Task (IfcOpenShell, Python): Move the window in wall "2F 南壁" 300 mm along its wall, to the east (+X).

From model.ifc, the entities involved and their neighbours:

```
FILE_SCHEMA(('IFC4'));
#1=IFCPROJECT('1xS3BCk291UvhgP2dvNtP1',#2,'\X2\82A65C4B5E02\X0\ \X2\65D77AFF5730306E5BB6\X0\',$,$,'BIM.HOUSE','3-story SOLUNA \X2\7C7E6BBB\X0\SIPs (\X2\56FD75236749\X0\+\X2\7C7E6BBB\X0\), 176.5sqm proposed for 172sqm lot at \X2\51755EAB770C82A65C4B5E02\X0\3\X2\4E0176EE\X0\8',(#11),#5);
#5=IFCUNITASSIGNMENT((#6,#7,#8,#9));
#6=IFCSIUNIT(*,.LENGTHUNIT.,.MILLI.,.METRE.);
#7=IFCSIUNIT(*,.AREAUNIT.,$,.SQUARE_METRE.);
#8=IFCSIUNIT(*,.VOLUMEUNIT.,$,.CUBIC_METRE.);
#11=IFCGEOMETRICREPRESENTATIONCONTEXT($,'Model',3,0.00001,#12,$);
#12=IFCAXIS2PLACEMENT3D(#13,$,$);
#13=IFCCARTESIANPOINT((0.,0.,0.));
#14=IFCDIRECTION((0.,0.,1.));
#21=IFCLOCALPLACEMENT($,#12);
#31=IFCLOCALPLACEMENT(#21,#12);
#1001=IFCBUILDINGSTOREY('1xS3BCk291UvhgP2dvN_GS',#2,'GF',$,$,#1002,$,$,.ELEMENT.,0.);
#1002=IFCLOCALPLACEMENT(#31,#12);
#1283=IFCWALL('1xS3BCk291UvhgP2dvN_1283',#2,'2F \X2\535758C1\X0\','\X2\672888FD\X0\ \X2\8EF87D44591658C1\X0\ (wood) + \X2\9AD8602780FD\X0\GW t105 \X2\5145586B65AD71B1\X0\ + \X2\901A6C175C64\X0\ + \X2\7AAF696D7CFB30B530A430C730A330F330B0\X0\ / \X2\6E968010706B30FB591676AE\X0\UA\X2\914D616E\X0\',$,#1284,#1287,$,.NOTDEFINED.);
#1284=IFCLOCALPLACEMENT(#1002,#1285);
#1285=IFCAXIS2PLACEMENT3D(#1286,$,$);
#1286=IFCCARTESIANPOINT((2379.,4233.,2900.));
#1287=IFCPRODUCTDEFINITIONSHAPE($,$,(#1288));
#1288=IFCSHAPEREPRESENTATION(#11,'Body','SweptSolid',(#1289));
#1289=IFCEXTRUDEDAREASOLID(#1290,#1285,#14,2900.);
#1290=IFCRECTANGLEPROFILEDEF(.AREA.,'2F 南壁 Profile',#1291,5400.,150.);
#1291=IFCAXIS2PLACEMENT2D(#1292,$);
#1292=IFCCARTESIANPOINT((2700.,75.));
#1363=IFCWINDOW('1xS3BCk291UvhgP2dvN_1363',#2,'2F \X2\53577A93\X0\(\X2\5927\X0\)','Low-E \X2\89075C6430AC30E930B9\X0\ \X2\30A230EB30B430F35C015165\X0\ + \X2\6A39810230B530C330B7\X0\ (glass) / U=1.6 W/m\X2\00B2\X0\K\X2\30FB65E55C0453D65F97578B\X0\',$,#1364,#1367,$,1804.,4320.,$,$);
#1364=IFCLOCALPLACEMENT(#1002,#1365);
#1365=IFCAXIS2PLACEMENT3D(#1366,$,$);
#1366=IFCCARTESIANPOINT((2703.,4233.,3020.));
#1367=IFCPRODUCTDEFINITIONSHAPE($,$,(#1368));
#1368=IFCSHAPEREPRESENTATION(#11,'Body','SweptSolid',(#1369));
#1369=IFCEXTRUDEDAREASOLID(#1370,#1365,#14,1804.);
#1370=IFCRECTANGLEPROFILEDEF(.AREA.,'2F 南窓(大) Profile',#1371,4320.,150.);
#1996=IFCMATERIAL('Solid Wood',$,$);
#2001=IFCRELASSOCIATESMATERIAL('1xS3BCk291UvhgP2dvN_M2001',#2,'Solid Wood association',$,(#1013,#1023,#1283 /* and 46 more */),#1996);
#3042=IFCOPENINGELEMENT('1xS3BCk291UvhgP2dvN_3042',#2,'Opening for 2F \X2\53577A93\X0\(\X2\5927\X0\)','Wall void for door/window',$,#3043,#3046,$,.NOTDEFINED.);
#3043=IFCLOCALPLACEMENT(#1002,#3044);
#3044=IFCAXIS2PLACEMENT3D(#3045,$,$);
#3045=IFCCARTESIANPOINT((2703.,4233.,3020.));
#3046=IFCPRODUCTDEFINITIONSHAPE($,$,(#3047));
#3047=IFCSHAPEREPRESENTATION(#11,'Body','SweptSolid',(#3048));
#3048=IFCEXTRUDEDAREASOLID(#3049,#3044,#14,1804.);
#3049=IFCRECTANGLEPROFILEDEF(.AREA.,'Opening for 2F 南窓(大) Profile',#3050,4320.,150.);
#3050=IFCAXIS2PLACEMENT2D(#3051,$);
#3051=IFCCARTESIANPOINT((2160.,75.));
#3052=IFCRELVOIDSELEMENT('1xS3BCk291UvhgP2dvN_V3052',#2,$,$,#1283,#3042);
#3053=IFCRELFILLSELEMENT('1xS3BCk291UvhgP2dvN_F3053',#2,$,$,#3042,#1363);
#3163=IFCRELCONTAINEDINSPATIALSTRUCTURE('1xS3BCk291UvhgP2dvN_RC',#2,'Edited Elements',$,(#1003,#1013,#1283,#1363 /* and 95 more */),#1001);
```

```python
import ifcopenshell
import ifcopenshell.api.geometry
import ifcopenshell.util.placement
import ifcopenshell.util.unit

model = ifcopenshell.open("model.ifc")
unit_scale = ifcopenshell.util.unit.calculate_unit_scale(model)

window = model.by_guid("1xS3BCk291UvhgP2dvN_1363")
opening = window.FillsVoids[0].RelatingOpeningElement
wall = opening.VoidsElements[0].RelatingBuildingElement

wall_matrix = ifcopenshell.util.placement.get_local_placement(wall.ObjectPlacement)
shift = wall_matrix[:3, 0] * 0.3 / unit_scale
before = ifcopenshell.util.placement.get_local_placement(window.ObjectPlacement)[:3, 3].copy()

# The window is not placed relative to its opening, so move both.
for product in (opening, window):
    matrix = ifcopenshell.util.placement.get_local_placement(product.ObjectPlacement)
    matrix[:3, 3] += shift
    ifcopenshell.api.geometry.edit_object_placement(model, product=product, matrix=matrix, is_si=False)

after = ifcopenshell.util.placement.get_local_placement(window.ObjectPlacement)[:3, 3]
print("window moved by", (after - before).round(3) + 0.0)

model.write("model_updated.ifc")
```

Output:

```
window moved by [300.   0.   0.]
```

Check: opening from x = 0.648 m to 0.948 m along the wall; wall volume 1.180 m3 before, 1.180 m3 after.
